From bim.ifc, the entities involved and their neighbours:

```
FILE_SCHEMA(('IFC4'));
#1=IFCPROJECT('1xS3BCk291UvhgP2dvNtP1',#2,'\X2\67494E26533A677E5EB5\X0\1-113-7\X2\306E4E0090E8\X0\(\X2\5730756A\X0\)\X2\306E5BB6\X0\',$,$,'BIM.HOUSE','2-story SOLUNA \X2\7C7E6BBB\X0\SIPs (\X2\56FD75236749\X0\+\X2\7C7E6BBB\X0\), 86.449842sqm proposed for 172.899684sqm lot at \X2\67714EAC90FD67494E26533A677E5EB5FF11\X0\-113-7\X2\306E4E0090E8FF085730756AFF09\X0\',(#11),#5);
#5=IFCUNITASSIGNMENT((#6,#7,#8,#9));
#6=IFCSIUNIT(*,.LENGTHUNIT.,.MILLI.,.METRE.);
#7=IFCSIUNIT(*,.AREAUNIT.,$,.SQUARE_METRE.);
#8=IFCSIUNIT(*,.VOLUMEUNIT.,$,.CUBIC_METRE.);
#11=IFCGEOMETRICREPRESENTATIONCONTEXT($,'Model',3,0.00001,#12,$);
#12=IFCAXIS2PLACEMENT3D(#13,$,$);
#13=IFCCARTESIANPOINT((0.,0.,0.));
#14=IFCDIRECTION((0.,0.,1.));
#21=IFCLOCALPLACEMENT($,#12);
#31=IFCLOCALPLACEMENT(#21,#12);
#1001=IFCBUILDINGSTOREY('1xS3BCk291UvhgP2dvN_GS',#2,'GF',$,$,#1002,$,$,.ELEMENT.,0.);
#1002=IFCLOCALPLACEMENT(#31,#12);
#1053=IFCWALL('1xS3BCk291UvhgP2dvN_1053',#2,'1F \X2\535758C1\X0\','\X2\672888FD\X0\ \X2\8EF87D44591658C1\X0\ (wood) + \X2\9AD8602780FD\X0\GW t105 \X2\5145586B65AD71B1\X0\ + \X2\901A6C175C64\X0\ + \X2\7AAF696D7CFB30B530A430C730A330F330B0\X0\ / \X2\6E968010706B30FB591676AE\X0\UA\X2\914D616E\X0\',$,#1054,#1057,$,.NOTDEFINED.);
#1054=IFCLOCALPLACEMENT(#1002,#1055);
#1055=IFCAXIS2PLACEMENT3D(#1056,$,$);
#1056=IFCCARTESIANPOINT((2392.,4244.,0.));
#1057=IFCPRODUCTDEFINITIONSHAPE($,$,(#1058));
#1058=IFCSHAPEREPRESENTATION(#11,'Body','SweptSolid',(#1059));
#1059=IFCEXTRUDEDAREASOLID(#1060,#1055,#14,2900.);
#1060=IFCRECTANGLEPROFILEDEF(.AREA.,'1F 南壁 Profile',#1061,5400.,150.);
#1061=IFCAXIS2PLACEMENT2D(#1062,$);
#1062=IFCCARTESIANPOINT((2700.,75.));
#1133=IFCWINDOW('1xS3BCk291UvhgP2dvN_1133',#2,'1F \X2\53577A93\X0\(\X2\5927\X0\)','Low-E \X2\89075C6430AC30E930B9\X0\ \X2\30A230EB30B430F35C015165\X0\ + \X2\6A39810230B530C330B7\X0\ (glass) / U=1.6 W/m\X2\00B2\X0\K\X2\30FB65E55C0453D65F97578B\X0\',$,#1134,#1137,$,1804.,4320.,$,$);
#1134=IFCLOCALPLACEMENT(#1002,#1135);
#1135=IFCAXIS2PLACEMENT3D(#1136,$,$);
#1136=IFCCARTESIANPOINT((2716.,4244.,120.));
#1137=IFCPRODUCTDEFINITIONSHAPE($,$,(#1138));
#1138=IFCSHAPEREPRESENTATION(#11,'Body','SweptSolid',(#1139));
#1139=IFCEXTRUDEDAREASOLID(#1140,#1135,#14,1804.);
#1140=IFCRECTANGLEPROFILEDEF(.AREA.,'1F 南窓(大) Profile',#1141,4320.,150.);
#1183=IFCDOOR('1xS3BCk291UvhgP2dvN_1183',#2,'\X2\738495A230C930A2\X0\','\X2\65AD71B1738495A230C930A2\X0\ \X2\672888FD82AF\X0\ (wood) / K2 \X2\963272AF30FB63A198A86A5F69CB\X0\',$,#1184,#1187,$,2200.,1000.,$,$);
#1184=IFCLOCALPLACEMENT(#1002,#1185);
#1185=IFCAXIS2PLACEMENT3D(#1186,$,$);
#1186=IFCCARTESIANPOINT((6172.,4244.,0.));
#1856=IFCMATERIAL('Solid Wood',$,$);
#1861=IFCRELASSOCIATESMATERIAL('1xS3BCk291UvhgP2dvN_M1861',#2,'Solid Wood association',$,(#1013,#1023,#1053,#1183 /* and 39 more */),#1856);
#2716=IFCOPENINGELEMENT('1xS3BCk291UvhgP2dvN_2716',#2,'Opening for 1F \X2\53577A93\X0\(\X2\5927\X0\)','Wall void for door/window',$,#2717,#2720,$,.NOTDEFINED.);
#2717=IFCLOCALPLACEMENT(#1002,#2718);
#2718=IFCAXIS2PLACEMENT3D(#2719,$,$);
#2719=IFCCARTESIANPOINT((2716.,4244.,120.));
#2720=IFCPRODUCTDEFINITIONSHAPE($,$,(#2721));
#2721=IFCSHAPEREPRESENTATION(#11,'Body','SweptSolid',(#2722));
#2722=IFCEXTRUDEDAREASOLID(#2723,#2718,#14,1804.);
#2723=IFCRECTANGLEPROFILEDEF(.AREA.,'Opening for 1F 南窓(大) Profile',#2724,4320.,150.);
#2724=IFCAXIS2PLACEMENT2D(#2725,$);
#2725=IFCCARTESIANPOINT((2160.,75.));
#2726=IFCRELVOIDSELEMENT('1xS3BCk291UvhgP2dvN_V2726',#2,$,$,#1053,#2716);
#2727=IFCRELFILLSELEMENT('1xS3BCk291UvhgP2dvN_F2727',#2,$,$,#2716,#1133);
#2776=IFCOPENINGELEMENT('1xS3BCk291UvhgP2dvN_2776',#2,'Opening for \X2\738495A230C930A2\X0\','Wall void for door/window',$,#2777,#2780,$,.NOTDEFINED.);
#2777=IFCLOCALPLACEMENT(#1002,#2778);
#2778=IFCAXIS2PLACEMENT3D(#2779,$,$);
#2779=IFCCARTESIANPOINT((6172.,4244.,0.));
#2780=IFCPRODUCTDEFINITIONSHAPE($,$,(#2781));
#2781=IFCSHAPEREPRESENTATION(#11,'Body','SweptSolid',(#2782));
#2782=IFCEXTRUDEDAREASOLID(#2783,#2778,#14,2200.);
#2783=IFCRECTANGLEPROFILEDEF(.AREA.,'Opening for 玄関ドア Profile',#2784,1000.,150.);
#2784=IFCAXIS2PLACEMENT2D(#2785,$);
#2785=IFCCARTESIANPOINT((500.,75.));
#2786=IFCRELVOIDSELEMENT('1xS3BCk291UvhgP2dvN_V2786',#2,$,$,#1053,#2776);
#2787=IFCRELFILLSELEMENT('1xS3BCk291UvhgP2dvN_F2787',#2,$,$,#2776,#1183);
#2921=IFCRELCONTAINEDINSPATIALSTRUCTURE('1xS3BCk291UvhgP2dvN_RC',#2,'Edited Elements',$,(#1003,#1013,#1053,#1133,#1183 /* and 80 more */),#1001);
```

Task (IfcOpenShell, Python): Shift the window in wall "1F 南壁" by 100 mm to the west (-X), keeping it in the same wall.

```python
import ifcopenshell
import ifcopenshell.api.geometry
import ifcopenshell.util.placement

model = ifcopenshell.open("bim.ifc")

window = model.by_id(1133)
opening = window.FillsVoids[0].RelatingOpeningElement
wall = opening.VoidsElements[0].RelatingBuildingElement

wall_matrix = ifcopenshell.util.placement.get_local_placement(wall.ObjectPlacement)
shift = wall_matrix[:3, 0] * -100.0
before = ifcopenshell.util.placement.get_local_placement(window.ObjectPlacement)[:3, 3].copy()

# The window is not placed relative to its opening, so move both.
for product in (opening, window):
    matrix = ifcopenshell.util.placement.get_local_placement(product.ObjectPlacement)
    matrix[:3, 3] += shift
    ifcopenshell.api.geometry.edit_object_placement(model, product=product, matrix=matrix, is_si=False)

after = ifcopenshell.util.placement.get_local_placement(window.ObjectPlacement)[:3, 3]
print("window moved by", (after - before).round(3) + 0.0)

model.write("bim_rev.ifc")
```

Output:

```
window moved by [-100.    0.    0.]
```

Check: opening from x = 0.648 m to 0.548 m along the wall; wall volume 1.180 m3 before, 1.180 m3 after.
